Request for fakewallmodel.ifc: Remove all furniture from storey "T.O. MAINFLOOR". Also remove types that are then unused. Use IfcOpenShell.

First a look at what the model holds.

```python
import ifcopenshell
import ifcopenshell.util.element

model = ifcopenshell.open("fakewallmodel.ifc")
print(model.schema)
storey = next(s for s in model.by_type("IfcBuildingStorey") if s.Name == "T.O. MAINFLOOR")
furniture = [e for e in ifcopenshell.util.element.get_decomposition(storey) if e.is_a("IfcFurnishingElement")]
seen = {}
for e in furniture:
    element_type = ifcopenshell.util.element.get_type(e)
    name = element_type.Name if element_type not in (None, e) else None
    seen[name] = seen.get(name, 0) + 1
for name, count in sorted(seen.items(), key=str):
    print(count, "x", name)
```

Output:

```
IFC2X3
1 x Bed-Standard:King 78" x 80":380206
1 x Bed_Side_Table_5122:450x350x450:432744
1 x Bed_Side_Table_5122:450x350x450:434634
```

```python
import ifcopenshell
import ifcopenshell.api.root
import ifcopenshell.util.element

model = ifcopenshell.open("fakewallmodel.ifc")

storey = next(s for s in model.by_type("IfcBuildingStorey") if s.Name == "T.O. MAINFLOOR")
furniture = [e for e in ifcopenshell.util.element.get_decomposition(storey) if e.is_a("IfcFurnishingElement")]
types = {ifcopenshell.util.element.get_type(e) for e in furniture} - {None, *furniture}

for e in furniture:
    ifcopenshell.api.root.remove_product(model, product=e)
print(len(furniture), "removed")

unused = [t for t in types if not ifcopenshell.util.element.get_types(t)]
for t in unused:
    ifcopenshell.api.root.remove_product(model, product=t)
print(len(unused), "unused types removed")

model.write("fakewallmodel_rev.ifc")
```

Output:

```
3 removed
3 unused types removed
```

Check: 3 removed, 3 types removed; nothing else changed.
